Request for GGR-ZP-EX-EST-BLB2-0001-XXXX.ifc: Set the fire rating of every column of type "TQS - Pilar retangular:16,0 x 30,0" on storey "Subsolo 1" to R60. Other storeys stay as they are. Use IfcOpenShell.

First a look at what the model holds.

```python
import ifcopenshell
import ifcopenshell.util.element

model = ifcopenshell.open("GGR-ZP-EX-EST-BLB2-0001-XXXX.ifc")
print(model.schema)
storey = next(s for s in model.by_type("IfcBuildingStorey") if s.Name == "Subsolo 1")
columns = [e for e in ifcopenshell.util.element.get_decomposition(storey) if e.is_a("IfcColumn")]
seen = {}
for e in columns:
    element_type = ifcopenshell.util.element.get_type(e)
    key = (element_type.Name if element_type != e and element_type else None, ifcopenshell.util.element.get_pset(e, "Pset_ColumnCommon", "FireRating"))
    seen[key] = seen.get(key, 0) + 1
for (name, value), count in sorted(seen.items(), key=str):
    print(count, "x", name, "|", value)
```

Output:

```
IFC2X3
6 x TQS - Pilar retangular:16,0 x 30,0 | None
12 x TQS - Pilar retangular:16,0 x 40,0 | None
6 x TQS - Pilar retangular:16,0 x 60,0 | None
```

```python
import ifcopenshell
import ifcopenshell.api.pset
import ifcopenshell.util.element

model = ifcopenshell.open("GGR-ZP-EX-EST-BLB2-0001-XXXX.ifc")

storey = next(s for s in model.by_type("IfcBuildingStorey") if s.Name == "Subsolo 1")
columns = [e for e in ifcopenshell.util.element.get_decomposition(storey) if e.is_a("IfcColumn")]

count = 0
for e in columns:
    element_type = ifcopenshell.util.element.get_type(e)
    if element_type in (None, e) or element_type.Name != "TQS - Pilar retangular:16,0 x 30,0":
        continue
    # add_pset returns the element's existing set when there is one.
    pset = ifcopenshell.api.pset.add_pset(model, product=e, name="Pset_ColumnCommon")
    ifcopenshell.api.pset.edit_pset(model, pset=pset, properties={"FireRating": "R60"})
    count += 1

print(count, "columns updated")

model.write("GGR-ZP-EX-EST-BLB2-0001-XXXX-out.ifc")
```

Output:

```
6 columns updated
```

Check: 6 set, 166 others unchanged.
